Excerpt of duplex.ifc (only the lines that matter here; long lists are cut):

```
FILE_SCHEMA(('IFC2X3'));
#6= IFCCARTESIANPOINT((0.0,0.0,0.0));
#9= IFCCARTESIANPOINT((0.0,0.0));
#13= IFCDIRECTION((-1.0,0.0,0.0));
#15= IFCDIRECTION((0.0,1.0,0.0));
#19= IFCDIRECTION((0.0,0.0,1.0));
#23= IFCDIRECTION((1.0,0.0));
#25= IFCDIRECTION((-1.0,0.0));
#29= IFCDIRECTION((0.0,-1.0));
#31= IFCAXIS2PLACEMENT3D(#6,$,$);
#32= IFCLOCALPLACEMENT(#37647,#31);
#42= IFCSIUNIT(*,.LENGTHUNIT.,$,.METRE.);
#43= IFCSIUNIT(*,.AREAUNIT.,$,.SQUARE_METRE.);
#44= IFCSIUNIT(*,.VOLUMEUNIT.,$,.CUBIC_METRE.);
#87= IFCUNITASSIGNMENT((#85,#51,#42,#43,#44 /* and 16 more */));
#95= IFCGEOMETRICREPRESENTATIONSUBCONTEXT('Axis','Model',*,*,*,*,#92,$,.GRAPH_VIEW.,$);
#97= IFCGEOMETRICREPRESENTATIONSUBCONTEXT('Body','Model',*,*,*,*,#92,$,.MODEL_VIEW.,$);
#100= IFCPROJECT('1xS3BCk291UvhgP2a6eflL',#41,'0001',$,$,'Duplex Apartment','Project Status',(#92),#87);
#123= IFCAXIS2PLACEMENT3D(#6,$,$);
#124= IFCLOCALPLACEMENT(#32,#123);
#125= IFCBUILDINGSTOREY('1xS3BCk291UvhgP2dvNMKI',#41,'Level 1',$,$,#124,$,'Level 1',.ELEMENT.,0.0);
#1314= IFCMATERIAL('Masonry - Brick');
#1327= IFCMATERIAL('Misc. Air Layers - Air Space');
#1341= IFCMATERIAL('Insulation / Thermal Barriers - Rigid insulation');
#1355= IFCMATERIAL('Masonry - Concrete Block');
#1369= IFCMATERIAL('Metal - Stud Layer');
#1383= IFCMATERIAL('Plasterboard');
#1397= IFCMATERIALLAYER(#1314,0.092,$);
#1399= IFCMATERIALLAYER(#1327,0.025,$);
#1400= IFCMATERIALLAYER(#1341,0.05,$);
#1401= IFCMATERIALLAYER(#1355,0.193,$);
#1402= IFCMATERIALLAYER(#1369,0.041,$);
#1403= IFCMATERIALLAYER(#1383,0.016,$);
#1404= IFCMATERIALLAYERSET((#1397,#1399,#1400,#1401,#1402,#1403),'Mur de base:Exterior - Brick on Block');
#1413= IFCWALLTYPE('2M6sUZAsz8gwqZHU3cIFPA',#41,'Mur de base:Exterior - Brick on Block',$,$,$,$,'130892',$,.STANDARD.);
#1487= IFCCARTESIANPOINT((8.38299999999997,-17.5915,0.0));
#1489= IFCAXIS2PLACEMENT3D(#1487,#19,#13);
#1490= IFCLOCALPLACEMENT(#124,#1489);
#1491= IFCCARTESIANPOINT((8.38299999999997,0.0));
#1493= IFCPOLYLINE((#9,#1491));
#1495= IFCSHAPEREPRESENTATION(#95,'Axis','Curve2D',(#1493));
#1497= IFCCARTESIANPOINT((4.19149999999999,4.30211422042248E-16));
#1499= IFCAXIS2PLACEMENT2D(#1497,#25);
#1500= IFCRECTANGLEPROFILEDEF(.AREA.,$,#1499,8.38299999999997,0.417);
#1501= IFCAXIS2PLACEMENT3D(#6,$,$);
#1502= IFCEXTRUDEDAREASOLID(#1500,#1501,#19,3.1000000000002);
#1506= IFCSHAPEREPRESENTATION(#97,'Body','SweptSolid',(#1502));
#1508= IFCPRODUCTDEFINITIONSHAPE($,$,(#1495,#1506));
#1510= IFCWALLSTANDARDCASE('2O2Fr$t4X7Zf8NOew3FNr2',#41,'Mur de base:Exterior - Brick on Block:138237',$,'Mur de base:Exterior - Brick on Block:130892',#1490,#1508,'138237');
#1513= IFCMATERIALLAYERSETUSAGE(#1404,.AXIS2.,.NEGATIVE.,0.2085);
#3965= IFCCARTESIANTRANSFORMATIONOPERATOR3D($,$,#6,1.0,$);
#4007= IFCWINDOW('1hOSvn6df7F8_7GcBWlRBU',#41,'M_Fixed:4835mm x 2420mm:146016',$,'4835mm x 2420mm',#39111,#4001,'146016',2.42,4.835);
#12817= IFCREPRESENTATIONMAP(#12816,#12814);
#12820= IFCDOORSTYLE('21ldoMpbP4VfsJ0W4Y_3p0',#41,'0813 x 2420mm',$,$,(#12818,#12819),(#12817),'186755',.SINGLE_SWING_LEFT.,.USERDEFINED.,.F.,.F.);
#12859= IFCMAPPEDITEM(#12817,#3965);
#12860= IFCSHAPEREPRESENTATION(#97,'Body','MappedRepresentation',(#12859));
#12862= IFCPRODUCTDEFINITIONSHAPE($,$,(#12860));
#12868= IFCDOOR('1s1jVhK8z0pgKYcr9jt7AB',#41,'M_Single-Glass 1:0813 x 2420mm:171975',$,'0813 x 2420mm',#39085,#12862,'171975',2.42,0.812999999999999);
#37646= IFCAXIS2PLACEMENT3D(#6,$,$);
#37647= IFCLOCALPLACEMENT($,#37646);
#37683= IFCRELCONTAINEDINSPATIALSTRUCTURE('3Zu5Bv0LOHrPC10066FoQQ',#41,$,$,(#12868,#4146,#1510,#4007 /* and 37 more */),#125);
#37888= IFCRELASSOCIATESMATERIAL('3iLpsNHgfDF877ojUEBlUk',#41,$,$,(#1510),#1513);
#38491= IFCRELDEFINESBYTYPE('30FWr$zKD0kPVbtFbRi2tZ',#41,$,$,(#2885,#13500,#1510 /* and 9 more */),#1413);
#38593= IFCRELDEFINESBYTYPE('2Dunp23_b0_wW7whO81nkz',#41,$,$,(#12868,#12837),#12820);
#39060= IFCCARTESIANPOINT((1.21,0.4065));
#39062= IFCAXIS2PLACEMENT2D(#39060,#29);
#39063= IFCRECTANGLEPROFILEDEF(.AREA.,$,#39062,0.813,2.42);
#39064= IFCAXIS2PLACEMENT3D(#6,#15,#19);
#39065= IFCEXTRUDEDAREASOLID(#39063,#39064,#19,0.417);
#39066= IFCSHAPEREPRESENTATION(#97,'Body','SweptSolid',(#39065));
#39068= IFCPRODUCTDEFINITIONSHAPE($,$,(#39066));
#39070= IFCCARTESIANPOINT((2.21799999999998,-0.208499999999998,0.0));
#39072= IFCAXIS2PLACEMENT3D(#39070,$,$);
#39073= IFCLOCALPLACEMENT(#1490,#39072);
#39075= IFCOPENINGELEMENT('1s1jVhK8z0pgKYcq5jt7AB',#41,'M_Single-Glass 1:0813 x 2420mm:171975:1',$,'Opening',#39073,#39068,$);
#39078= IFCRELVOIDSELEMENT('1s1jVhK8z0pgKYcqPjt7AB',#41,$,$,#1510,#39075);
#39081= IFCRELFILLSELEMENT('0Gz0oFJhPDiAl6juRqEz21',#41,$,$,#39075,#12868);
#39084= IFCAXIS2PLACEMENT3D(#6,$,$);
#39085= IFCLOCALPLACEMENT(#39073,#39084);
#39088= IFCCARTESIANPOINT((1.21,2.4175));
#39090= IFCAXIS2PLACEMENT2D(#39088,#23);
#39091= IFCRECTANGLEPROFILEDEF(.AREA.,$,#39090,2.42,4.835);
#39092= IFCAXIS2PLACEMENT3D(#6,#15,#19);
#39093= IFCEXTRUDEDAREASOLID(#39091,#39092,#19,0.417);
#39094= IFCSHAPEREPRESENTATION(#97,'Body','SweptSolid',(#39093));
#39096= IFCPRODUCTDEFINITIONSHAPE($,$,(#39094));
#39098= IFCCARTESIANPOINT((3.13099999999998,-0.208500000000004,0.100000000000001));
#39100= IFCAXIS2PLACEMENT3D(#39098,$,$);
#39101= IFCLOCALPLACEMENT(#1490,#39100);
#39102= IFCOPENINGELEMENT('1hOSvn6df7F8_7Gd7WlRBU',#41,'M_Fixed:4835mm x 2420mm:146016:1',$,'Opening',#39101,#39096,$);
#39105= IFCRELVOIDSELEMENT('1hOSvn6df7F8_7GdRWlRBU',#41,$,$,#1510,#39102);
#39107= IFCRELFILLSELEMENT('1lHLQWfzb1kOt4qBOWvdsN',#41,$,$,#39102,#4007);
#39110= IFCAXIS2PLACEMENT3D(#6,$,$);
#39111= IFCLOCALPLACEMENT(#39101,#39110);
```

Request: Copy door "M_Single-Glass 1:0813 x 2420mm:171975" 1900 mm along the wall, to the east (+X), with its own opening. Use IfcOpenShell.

```python
import ifcopenshell
import ifcopenshell.api.feature
import ifcopenshell.api.geometry
import ifcopenshell.api.root
import ifcopenshell.geom
import ifcopenshell.util.element
import ifcopenshell.util.placement
import ifcopenshell.util.shape

model = ifcopenshell.open("duplex.ifc")
settings = ifcopenshell.geom.settings()


def volume(element):
    """Net volume in cubic metres, openings subtracted."""
    shape = ifcopenshell.geom.create_shape(settings, element)
    return ifcopenshell.util.shape.get_volume(shape.geometry)


def reuse_history(source, copy):
    """copy_class also copies each property set's owner history, people and application; keep the originals."""
    for rel in copy.IsDefinedBy:
        if rel.is_a("IfcRelDefinesByProperties") and (history := rel.RelatingPropertyDefinition.OwnerHistory):
            rel.RelatingPropertyDefinition.OwnerHistory = source.OwnerHistory
            ifcopenshell.util.element.remove_deep2(model, history)


door = model.by_id(12868)
opening = door.FillsVoids[0].RelatingOpeningElement
wall = opening.VoidsElements[0].RelatingBuildingElement
before = volume(wall)
shift = ifcopenshell.util.placement.get_local_placement(wall.ObjectPlacement)[:3, 0] * -1.9

# copy_class copies the void relationship, type, container and properties, but no geometry.
new_opening = ifcopenshell.api.root.copy_class(model, product=opening)
new_opening.Representation = ifcopenshell.util.element.copy_deep(
    model, opening.Representation, exclude=["IfcGeometricRepresentationContext", "IfcRepresentationMap"]
)
new_opening.Name = "M_Single-Glass 1:0813 x 2420mm"
new_door = ifcopenshell.api.root.copy_class(model, product=door)
new_door.Representation = ifcopenshell.util.element.copy_deep(
    model, door.Representation, exclude=["IfcGeometricRepresentationContext", "IfcRepresentationMap"]
)
new_door.Name = "M_Single-Glass 1:0813 x 2420mm"
new_door.Tag = None
reuse_history(door, new_door)
fills = ifcopenshell.api.feature.add_filling(model, opening=new_opening, element=new_door)
fills.OwnerHistory = new_door.OwnerHistory  # required in IFC2X3

for old, new in ((opening, new_opening), (door, new_door)):
    matrix = ifcopenshell.util.placement.get_local_placement(old.ObjectPlacement)
    matrix[:3, 3] += shift
    ifcopenshell.api.geometry.edit_object_placement(model, product=new, matrix=matrix, is_si=False)

after = volume(wall)

print(f"wall volume {before:.3f} -> {after:.3f} m3")

model.write("duplex_edited.ifc")
```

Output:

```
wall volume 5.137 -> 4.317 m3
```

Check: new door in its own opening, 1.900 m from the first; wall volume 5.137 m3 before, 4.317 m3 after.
